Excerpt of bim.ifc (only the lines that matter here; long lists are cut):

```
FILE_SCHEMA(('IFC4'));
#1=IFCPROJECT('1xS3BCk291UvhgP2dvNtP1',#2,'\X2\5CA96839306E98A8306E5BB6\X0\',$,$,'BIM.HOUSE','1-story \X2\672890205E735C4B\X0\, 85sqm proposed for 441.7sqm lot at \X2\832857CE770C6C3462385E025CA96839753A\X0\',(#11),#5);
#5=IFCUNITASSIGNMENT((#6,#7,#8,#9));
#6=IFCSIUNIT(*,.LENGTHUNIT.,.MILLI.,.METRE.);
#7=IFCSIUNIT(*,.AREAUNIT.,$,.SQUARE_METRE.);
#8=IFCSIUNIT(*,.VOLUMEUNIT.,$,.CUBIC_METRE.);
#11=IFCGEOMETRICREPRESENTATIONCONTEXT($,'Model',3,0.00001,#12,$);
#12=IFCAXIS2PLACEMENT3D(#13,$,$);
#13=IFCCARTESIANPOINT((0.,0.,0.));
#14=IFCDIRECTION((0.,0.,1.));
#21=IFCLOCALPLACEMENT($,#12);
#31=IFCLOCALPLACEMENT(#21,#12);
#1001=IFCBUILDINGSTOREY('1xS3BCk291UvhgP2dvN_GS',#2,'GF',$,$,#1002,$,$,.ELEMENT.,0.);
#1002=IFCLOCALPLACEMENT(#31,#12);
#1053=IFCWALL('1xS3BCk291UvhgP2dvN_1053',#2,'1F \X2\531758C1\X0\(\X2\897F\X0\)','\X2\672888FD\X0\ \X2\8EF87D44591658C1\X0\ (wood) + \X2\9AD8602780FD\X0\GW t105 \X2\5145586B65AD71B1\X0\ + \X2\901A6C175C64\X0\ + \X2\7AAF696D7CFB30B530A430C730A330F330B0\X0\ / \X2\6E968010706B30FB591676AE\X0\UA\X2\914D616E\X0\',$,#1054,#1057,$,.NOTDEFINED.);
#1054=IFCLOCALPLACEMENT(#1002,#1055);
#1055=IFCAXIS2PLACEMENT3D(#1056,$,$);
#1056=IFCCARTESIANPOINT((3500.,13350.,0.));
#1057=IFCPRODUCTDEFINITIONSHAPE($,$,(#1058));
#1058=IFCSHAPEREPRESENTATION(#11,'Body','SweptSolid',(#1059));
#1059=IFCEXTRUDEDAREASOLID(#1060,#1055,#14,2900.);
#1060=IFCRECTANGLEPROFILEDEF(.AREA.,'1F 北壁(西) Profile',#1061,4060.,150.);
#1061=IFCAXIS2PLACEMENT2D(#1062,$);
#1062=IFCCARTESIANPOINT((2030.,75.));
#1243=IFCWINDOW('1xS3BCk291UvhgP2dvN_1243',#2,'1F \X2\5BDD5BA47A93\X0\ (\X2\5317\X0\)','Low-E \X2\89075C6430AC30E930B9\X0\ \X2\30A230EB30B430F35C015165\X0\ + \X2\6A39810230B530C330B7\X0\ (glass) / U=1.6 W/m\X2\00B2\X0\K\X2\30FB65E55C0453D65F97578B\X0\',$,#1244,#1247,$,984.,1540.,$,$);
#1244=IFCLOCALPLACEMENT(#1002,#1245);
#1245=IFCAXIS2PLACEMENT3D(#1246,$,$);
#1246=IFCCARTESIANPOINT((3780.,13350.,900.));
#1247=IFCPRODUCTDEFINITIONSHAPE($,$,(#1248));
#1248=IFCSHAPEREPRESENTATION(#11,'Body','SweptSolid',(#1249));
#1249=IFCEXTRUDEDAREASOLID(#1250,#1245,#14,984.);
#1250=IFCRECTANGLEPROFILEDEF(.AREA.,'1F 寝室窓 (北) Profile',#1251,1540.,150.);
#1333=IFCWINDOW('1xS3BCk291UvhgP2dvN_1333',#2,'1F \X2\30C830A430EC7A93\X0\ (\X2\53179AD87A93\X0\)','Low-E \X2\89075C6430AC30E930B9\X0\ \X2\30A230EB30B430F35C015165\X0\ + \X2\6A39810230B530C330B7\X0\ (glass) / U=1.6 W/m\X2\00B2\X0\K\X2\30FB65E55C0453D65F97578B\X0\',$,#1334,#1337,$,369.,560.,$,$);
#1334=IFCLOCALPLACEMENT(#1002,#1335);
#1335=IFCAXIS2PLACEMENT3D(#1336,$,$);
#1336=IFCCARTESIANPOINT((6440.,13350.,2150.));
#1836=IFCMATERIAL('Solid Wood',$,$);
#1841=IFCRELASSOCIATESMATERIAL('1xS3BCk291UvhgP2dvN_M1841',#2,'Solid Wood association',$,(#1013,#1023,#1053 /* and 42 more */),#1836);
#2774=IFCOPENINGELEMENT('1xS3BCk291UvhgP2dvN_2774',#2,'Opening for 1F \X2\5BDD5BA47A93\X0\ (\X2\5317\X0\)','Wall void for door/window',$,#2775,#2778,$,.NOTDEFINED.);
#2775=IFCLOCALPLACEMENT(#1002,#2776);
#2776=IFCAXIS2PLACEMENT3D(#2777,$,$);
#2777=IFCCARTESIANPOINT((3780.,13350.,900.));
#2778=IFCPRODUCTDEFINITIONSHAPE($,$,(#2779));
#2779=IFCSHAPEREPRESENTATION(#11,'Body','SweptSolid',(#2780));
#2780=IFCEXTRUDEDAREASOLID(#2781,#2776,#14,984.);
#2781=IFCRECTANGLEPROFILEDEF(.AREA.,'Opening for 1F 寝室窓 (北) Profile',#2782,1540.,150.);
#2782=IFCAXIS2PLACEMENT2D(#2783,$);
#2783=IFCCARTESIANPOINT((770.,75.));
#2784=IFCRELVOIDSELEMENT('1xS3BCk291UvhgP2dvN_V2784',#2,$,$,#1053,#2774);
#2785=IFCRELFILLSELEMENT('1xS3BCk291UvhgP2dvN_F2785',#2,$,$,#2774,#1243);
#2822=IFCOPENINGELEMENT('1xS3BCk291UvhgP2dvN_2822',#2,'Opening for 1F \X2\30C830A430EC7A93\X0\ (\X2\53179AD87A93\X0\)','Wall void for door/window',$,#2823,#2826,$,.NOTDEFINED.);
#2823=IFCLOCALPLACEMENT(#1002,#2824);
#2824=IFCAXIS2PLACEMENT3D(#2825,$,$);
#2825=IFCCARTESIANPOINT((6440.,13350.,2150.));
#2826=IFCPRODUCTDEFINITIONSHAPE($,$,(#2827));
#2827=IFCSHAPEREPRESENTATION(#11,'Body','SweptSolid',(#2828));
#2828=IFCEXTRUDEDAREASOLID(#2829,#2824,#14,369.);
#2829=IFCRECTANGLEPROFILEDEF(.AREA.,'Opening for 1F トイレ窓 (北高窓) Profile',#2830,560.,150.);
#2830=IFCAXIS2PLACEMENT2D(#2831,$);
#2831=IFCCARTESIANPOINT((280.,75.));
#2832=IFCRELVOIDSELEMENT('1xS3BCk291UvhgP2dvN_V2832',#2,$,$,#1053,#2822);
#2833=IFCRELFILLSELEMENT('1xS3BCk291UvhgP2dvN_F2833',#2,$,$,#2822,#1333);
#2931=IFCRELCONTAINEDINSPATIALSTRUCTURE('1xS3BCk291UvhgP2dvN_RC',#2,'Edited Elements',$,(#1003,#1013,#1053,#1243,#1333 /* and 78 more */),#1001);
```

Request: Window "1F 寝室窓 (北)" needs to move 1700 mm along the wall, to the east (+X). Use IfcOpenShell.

```python
import ifcopenshell
import ifcopenshell.api.geometry
import ifcopenshell.util.placement
import ifcopenshell.util.unit

model = ifcopenshell.open("bim.ifc")
unit_scale = ifcopenshell.util.unit.calculate_unit_scale(model)

window = model.by_guid("1xS3BCk291UvhgP2dvN_1243")
opening = window.FillsVoids[0].RelatingOpeningElement
wall = opening.VoidsElements[0].RelatingBuildingElement

wall_matrix = ifcopenshell.util.placement.get_local_placement(wall.ObjectPlacement)
shift = wall_matrix[:3, 0] * 1.7 / unit_scale
before = ifcopenshell.util.placement.get_local_placement(window.ObjectPlacement)[:3, 3].copy()

# The window is not placed relative to its opening, so move both.
for product in (opening, window):
    matrix = ifcopenshell.util.placement.get_local_placement(product.ObjectPlacement)
    matrix[:3, 3] += shift
    ifcopenshell.api.geometry.edit_object_placement(model, product=product, matrix=matrix, is_si=False)

after = ifcopenshell.util.placement.get_local_placement(window.ObjectPlacement)[:3, 3]
print("window moved by", (after - before).round(3) + 0.0)

model.write("bim_edited.ifc")
```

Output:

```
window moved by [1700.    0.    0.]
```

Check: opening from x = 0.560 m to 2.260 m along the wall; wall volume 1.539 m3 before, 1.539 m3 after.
